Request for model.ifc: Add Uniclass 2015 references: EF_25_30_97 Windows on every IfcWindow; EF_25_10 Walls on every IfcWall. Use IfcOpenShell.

First a look at what the model holds.

```python
import ifcopenshell

model = ifcopenshell.open("model.ifc")
print(model.schema)
print("classifications:", [c.Name for c in model.by_type("IfcClassification")])
for ifc_class in ("IfcDoor", "IfcRoof", "IfcStair", "IfcWall", "IfcWindow"):
    print(ifc_class, len(model.by_type(ifc_class)))
```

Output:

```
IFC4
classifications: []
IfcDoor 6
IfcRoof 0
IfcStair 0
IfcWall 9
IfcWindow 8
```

```python
import ifcopenshell
import ifcopenshell.api.classification

model = ifcopenshell.open("model.ifc")

system = ifcopenshell.api.classification.add_classification(model, classification="Uniclass 2015")

codes = {
    "IfcWindow": ("EF_25_30_97", "Windows"),
    "IfcWall": ("EF_25_10", "Walls"),
}
for ifc_class, (code, name) in codes.items():
    products = model.by_type(ifc_class)
    ifcopenshell.api.classification.add_reference(
        model, products=products, classification=system, identification=code, name=name
    )
    print(code, len(products))

model.write("model_v2.ifc")
```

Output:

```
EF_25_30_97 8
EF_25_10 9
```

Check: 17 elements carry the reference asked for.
